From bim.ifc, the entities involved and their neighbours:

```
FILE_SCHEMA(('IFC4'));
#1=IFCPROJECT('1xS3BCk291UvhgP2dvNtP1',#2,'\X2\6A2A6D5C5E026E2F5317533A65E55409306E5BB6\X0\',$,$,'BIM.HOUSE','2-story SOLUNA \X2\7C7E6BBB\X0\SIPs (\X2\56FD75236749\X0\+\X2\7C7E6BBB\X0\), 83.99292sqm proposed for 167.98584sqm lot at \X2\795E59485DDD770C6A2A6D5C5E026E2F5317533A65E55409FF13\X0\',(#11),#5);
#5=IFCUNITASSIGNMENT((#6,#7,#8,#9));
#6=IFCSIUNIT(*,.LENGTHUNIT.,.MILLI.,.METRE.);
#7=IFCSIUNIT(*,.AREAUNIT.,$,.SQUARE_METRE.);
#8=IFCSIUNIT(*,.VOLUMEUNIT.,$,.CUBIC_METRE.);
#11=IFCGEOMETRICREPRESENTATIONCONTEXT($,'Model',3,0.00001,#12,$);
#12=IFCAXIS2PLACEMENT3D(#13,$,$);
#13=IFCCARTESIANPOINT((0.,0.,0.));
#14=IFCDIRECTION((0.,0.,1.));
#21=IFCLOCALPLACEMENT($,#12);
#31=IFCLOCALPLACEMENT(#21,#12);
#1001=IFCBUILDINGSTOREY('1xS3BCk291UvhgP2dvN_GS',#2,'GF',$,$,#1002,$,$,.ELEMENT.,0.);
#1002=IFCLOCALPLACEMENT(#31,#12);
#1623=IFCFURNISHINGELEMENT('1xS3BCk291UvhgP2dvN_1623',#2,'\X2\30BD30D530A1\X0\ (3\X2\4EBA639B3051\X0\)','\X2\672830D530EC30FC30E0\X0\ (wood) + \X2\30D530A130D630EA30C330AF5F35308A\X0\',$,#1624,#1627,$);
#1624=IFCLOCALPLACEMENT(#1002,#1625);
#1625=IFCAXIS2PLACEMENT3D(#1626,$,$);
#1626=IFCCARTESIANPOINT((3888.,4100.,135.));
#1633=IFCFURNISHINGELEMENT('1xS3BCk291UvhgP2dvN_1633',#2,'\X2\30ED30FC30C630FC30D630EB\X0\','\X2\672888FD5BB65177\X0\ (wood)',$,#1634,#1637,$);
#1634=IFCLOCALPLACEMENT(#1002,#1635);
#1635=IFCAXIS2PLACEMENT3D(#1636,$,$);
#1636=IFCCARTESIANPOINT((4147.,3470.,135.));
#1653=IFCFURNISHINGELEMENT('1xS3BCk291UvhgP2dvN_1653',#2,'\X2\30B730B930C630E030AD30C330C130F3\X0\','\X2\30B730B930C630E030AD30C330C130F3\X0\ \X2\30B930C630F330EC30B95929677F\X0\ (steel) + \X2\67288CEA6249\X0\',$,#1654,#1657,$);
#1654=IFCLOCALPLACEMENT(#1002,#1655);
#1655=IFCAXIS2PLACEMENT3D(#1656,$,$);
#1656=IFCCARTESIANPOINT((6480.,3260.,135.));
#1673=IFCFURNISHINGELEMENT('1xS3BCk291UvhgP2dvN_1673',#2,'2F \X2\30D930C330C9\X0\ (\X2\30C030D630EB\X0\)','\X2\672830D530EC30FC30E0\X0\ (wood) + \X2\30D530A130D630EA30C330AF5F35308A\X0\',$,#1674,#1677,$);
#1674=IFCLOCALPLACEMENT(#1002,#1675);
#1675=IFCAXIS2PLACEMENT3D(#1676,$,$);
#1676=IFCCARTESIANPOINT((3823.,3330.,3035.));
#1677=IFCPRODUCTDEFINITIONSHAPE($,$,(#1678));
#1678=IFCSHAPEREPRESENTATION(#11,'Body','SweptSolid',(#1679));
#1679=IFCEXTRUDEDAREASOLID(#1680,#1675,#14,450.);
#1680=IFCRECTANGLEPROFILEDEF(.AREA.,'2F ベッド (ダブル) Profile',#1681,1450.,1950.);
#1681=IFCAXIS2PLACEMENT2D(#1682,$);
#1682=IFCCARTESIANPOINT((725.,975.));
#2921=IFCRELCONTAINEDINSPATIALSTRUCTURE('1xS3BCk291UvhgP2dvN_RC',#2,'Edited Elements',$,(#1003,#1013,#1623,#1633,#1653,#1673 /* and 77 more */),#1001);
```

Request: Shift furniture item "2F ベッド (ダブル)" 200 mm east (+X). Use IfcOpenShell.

```python
import ifcopenshell
import ifcopenshell.api.geometry
import ifcopenshell.util.placement
import ifcopenshell.util.unit

model = ifcopenshell.open("bim.ifc")
unit_scale = ifcopenshell.util.unit.calculate_unit_scale(model)

item = model.by_id(1673)
matrix = ifcopenshell.util.placement.get_local_placement(item.ObjectPlacement)
matrix[0, 3] += 0.2 / unit_scale
ifcopenshell.api.geometry.edit_object_placement(model, product=item, matrix=matrix, is_si=False)

print(ifcopenshell.util.placement.get_local_placement(item.ObjectPlacement).round(3) + 0.0)

model.write("bim-out.ifc")
```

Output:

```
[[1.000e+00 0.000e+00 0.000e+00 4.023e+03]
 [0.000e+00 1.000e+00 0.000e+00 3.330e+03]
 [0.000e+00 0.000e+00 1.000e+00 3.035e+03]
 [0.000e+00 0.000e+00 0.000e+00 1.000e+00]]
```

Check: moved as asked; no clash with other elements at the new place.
